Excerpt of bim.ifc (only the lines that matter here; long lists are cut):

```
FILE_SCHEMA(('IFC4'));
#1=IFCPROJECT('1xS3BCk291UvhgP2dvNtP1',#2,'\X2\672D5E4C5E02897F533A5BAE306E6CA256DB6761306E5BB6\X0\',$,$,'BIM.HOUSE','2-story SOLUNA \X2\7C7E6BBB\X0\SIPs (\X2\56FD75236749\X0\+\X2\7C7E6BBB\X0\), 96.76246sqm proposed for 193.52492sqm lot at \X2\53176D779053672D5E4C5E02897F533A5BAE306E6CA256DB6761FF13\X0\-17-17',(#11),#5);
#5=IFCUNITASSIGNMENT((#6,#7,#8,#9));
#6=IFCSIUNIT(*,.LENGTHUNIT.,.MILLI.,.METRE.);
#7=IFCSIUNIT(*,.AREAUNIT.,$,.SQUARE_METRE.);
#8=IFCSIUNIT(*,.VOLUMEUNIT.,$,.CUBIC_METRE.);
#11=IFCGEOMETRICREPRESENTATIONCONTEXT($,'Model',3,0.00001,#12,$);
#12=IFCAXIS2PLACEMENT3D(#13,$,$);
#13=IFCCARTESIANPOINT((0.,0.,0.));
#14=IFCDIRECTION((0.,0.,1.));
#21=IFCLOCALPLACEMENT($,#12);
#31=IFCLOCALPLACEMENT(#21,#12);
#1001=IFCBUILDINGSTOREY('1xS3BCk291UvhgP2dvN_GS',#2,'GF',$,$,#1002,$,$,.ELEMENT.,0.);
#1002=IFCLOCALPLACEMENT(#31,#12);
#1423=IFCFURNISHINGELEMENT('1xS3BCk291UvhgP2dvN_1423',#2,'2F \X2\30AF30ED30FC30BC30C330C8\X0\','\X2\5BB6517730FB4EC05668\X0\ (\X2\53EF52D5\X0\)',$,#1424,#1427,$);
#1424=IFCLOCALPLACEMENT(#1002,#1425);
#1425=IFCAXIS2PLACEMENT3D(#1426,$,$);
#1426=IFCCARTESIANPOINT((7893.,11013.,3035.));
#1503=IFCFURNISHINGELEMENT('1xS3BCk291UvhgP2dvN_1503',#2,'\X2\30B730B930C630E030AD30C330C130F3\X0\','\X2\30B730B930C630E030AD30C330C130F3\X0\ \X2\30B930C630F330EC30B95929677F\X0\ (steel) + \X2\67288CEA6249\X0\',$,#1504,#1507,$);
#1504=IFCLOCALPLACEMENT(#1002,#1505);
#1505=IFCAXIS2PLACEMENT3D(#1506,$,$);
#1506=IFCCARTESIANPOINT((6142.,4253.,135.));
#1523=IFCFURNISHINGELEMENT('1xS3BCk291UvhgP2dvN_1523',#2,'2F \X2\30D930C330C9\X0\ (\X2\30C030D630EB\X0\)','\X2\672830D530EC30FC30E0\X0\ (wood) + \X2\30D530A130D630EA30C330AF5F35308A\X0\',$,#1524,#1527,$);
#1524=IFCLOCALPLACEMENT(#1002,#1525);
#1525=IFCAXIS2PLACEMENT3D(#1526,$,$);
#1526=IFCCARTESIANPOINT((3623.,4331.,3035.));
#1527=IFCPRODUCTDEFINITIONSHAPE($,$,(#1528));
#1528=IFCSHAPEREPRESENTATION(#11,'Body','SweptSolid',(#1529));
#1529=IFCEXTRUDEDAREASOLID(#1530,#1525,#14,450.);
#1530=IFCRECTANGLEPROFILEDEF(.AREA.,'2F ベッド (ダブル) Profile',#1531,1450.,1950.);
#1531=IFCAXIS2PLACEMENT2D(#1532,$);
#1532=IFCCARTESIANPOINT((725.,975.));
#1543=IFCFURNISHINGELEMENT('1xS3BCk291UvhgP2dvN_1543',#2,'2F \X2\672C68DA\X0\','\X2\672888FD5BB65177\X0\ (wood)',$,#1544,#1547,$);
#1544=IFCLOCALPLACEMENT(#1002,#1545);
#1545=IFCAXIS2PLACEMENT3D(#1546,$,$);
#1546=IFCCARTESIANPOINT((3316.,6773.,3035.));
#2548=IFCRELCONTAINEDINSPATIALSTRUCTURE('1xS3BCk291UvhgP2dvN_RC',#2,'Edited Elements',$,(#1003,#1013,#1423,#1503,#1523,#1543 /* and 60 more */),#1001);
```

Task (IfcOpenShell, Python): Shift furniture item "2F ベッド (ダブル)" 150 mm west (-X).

```python
import ifcopenshell
import ifcopenshell.api.geometry
import ifcopenshell.util.placement
import ifcopenshell.util.unit

model = ifcopenshell.open("bim.ifc")
unit_scale = ifcopenshell.util.unit.calculate_unit_scale(model)

item = model.by_guid("1xS3BCk291UvhgP2dvN_1523")
matrix = ifcopenshell.util.placement.get_local_placement(item.ObjectPlacement)
matrix[0, 3] -= 0.15 / unit_scale
ifcopenshell.api.geometry.edit_object_placement(model, product=item, matrix=matrix, is_si=False)

print(ifcopenshell.util.placement.get_local_placement(item.ObjectPlacement).round(3) + 0.0)

model.write("bim-out.ifc")
```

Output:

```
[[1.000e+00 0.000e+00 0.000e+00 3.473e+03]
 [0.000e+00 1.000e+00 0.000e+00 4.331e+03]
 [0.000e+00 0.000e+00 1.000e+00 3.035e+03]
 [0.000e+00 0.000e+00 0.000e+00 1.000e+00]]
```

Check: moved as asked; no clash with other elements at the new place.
